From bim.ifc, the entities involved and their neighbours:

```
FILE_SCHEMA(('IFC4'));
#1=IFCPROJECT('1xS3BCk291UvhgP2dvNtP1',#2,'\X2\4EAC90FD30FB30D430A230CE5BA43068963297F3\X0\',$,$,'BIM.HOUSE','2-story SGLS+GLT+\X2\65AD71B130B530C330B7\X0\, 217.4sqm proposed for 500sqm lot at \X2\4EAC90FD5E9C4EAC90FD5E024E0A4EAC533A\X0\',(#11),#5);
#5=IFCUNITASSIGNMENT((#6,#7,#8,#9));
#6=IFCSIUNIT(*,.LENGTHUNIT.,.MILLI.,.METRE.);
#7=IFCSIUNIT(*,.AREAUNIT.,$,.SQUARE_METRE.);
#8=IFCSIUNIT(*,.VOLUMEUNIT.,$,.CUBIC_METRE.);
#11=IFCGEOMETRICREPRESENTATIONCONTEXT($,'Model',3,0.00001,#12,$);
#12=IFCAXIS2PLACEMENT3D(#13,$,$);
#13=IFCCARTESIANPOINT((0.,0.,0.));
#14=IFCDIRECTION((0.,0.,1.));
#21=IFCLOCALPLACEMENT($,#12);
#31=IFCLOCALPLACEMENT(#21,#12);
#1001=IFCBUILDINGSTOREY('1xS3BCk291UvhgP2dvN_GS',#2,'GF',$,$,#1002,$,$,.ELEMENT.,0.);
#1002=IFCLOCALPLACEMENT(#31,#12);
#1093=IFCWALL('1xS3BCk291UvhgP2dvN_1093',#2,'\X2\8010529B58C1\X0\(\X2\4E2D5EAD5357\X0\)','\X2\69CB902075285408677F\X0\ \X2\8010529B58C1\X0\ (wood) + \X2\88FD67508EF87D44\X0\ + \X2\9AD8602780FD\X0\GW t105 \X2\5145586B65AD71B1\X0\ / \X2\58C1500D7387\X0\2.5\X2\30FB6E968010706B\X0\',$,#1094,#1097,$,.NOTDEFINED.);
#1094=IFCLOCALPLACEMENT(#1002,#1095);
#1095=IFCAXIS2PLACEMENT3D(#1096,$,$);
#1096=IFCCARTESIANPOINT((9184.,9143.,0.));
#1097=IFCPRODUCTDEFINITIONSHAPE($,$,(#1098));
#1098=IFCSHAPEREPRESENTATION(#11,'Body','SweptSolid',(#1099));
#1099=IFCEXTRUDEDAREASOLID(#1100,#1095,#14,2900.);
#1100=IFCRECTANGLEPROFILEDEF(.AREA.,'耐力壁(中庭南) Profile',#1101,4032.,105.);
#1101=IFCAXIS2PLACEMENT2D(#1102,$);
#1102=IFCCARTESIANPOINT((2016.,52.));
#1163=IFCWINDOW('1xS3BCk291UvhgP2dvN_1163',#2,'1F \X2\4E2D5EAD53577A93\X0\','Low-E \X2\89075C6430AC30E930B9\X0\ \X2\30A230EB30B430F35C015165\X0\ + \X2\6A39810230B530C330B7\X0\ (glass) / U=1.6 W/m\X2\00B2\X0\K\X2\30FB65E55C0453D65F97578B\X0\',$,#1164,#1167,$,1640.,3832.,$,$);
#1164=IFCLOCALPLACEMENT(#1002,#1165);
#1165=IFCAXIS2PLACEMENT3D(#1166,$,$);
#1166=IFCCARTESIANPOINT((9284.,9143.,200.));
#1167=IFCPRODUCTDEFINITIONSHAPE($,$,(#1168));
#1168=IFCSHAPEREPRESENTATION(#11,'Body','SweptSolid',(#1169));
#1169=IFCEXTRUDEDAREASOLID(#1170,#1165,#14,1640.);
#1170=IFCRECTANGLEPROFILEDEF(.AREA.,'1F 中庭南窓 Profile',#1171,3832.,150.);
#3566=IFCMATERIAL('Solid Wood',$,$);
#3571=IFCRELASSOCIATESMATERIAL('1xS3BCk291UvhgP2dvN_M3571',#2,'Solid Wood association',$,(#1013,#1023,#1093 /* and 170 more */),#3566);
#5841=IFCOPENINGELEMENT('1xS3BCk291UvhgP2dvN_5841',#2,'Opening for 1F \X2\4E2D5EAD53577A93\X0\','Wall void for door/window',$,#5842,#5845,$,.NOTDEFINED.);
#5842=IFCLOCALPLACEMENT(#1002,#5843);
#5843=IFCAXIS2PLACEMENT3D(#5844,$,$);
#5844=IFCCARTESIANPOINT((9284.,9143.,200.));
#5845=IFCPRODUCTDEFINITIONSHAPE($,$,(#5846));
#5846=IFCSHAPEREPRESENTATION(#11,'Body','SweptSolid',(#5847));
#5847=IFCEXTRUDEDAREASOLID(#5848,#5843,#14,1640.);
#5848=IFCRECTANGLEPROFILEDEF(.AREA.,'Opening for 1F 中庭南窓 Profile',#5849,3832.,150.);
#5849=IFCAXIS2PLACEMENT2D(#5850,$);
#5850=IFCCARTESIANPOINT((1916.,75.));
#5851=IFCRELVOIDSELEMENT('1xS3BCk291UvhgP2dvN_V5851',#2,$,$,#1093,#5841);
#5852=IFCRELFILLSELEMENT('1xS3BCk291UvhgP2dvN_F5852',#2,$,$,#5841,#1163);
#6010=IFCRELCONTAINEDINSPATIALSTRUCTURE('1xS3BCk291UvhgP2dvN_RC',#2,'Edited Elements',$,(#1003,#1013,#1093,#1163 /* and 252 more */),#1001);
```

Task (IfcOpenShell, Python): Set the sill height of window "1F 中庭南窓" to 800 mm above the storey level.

```python
import numpy as np
import ifcopenshell
import ifcopenshell.api.geometry
import ifcopenshell.geom
import ifcopenshell.util.element
import ifcopenshell.util.placement
import ifcopenshell.util.shape
import ifcopenshell.util.unit

model = ifcopenshell.open("bim.ifc")
unit_scale = ifcopenshell.util.unit.calculate_unit_scale(model)

window = model.by_guid("1xS3BCk291UvhgP2dvN_1163")
opening = window.FillsVoids[0].RelatingOpeningElement
storey = ifcopenshell.util.element.get_container(window, ifc_class="IfcBuildingStorey")
level = ifcopenshell.util.placement.get_local_placement(storey.ObjectPlacement)[2, 3]

# The opening's origin need not be at the sill, so measure its lowest point.
shape = ifcopenshell.geom.create_shape(ifcopenshell.geom.settings(), opening)
bottom = ifcopenshell.util.shape.get_shape_bottom_elevation(shape, shape.geometry) / unit_scale
dz = level + 0.8 / unit_scale - bottom

shift = np.array([0.0, 0.0, dz])
# The window is not placed relative to its opening, so move both.
for product in (opening, window):
    matrix = ifcopenshell.util.placement.get_local_placement(product.ObjectPlacement)
    matrix[:3, 3] += shift
    ifcopenshell.api.geometry.edit_object_placement(model, product=product, matrix=matrix, is_si=False)

print(f"moved by {dz * unit_scale:+.3f} m")

model.write("bim_updated.ifc")
```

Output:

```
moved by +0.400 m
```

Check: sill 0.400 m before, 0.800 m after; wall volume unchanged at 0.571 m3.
